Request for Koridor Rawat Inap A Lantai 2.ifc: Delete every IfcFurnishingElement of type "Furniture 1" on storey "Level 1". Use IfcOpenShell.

First a look at what the model holds.

```python
import ifcopenshell
import ifcopenshell.util.element

model = ifcopenshell.open("Koridor Rawat Inap A Lantai 2.ifc")
print(model.schema)
storey = next(s for s in model.by_type("IfcBuildingStorey") if s.Name == "Level 1")
furniture = [e for e in ifcopenshell.util.element.get_decomposition(storey) if e.is_a("IfcFurnishingElement")]
seen = {}
for e in furniture:
    element_type = ifcopenshell.util.element.get_type(e)
    name = element_type.Name if element_type not in (None, e) else None
    seen[name] = seen.get(name, 0) + 1
for name, count in sorted(seen.items(), key=str):
    print(count, "x", name)
```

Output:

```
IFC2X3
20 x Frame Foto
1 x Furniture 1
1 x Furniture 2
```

```python
import ifcopenshell
import ifcopenshell.api.root
import ifcopenshell.util.element

model = ifcopenshell.open("Koridor Rawat Inap A Lantai 2.ifc")

storey = next(s for s in model.by_type("IfcBuildingStorey") if s.Name == "Level 1")
furniture = [e for e in ifcopenshell.util.element.get_decomposition(storey) if e.is_a("IfcFurnishingElement")]
targets = [e for e in furniture if (t := ifcopenshell.util.element.get_type(e)) not in (None, e) and t.Name == "Furniture 1"]

for e in targets:
    ifcopenshell.api.root.remove_product(model, product=e)
print(len(targets), "removed")

model.write("Koridor Rawat Inap A Lantai 2_v2.ifc")
```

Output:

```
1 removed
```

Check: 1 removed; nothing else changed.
